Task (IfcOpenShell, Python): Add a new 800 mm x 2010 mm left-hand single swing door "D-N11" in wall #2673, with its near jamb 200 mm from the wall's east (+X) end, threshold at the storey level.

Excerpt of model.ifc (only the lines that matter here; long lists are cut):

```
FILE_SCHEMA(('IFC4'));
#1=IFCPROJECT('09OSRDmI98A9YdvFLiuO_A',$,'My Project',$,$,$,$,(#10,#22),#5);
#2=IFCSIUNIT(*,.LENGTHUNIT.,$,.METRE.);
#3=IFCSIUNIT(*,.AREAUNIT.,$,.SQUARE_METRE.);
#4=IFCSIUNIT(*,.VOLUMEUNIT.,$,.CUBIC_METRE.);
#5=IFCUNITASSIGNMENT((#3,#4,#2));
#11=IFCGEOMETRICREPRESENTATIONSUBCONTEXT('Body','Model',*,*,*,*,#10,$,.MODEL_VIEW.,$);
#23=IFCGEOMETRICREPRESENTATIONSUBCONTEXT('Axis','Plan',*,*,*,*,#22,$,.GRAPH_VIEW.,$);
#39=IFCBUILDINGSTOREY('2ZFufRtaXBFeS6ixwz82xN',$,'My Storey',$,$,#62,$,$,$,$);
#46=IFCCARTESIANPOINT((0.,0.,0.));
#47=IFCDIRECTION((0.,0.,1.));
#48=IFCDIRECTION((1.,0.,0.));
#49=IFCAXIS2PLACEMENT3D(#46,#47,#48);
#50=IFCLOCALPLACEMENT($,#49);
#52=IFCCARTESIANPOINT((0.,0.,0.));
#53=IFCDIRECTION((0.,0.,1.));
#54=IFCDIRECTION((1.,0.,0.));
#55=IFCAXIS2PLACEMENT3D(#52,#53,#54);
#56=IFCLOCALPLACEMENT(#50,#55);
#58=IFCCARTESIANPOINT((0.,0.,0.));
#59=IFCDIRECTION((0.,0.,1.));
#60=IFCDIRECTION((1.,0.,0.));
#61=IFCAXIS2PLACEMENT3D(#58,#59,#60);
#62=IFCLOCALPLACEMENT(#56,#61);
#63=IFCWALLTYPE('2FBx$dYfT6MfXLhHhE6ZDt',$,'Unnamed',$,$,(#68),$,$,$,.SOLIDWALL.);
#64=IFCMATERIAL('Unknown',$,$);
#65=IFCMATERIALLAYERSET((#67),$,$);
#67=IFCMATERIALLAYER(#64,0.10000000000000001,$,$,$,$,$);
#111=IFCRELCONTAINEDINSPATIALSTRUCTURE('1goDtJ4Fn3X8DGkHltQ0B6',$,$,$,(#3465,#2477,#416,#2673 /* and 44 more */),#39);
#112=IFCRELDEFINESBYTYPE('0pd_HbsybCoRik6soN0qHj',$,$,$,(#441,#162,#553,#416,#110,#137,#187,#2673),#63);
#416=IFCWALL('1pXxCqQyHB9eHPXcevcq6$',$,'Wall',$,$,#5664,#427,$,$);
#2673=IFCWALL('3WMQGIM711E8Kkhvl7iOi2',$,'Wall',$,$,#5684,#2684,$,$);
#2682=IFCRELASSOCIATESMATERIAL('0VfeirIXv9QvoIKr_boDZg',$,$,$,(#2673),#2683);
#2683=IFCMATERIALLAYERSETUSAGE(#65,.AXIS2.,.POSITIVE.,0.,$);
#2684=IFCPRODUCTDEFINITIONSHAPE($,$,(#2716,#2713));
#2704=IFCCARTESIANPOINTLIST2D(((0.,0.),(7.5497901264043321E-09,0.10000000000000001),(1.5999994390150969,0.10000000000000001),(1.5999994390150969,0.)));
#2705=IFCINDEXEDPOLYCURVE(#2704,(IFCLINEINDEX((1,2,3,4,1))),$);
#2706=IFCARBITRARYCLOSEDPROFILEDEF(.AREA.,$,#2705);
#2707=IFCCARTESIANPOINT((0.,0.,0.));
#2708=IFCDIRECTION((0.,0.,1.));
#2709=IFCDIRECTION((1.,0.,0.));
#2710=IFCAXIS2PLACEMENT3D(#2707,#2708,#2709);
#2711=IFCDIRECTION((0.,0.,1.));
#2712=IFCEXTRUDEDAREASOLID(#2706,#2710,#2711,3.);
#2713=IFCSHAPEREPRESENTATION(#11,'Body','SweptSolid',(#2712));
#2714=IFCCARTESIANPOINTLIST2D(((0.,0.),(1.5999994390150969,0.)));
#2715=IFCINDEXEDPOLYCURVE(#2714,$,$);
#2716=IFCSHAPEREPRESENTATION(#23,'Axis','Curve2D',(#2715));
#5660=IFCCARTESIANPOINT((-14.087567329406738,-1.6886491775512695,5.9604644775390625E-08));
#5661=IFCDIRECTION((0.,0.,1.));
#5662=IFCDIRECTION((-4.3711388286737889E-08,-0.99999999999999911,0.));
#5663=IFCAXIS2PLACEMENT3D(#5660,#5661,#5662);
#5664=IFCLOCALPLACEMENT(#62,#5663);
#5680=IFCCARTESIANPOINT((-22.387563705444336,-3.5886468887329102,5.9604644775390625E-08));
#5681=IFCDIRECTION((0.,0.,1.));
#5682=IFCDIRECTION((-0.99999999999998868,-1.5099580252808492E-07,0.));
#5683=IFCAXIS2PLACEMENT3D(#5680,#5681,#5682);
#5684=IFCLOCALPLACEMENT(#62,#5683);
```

```python
import numpy as np
import ifcopenshell
import ifcopenshell.api.feature
import ifcopenshell.api.geometry
import ifcopenshell.api.root
import ifcopenshell.api.spatial
import ifcopenshell.geom
import ifcopenshell.util.element
import ifcopenshell.util.placement
import ifcopenshell.util.representation
import ifcopenshell.util.shape
import ifcopenshell.util.unit

model = ifcopenshell.open("model.ifc")
unit_scale = ifcopenshell.util.unit.calculate_unit_scale(model)
settings = ifcopenshell.geom.settings()


def volume(element):
    """Net volume in cubic metres, openings subtracted."""
    shape = ifcopenshell.geom.create_shape(settings, element)
    return ifcopenshell.util.shape.get_volume(shape.geometry)


wall = model.by_id(2673)
storey = ifcopenshell.util.element.get_container(wall, ifc_class="IfcBuildingStorey")
context = ifcopenshell.util.representation.get_context(model, "Model", "Body", "MODEL_VIEW")
before = volume(wall)

width, height, from_end, sill = 0.8, 2.01, 0.2, 0.0  # metres

# The wall runs along its own X axis, and the end named is its -X end.
wall_shape = ifcopenshell.geom.create_shape(settings, wall)
x, y, z = ifcopenshell.util.shape.get_vertices(wall_shape.geometry).T
start = x.min() + from_end
face, thickness = float(y.min()), float(y.max() - y.min())
wall_matrix = ifcopenshell.util.placement.get_local_placement(wall.ObjectPlacement)
level = ifcopenshell.util.placement.get_local_placement(storey.ObjectPlacement)[2, 3]


def in_wall(x, y):
    """Placement at x, y metres in the wall's axes, at sill height."""
    matrix = wall_matrix.copy()
    matrix[:, 3] = wall_matrix @ np.array([x / unit_scale, y / unit_scale, 0.0, 1.0])
    matrix[2, 3] = level + sill / unit_scale
    return matrix


# Opening: a box that overshoots both wall faces by 50 mm.
opening = ifcopenshell.api.root.create_entity(model, ifc_class="IfcOpeningElement", predefined_type="OPENING")
box = ifcopenshell.api.geometry.add_wall_representation(
    model, context=context, length=width, height=height, thickness=thickness + 0.1
)
ifcopenshell.api.geometry.assign_representation(model, product=opening, representation=box)
ifcopenshell.api.geometry.edit_object_placement(model, product=opening, matrix=in_wall(start, face - 0.05), is_si=False)
ifcopenshell.api.feature.add_feature(model, feature=opening, element=wall)

door = ifcopenshell.api.root.create_entity(model, ifc_class="IfcDoor", name="D-N11", predefined_type="DOOR")
door.OverallWidth, door.OverallHeight = width / unit_scale, height / unit_scale
door.OperationType = "SINGLE_SWING_LEFT"
body = ifcopenshell.api.geometry.add_door_representation(
    model,
    context=context,
    overall_width=door.OverallWidth,
    overall_height=door.OverallHeight,
    operation_type="SINGLE_SWING_LEFT",
    lining_properties={"LiningDepth": thickness / unit_scale, "ThresholdDepth": thickness / unit_scale},
)
ifcopenshell.api.geometry.assign_representation(model, product=door, representation=body)
ifcopenshell.api.spatial.assign_container(model, products=[door], relating_structure=storey)
ifcopenshell.api.feature.add_filling(model, opening=opening, element=door)

# The lining spans the wall, so the door starts at the wall face.
ifcopenshell.api.geometry.edit_object_placement(model, product=door, matrix=in_wall(start, face), is_si=False)

after = volume(wall)

print(f"wall volume {before:.3f} -> {after:.3f} m3")

model.write("model_updated.ifc")
```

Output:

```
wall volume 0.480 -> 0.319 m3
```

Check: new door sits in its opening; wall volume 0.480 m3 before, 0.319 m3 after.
